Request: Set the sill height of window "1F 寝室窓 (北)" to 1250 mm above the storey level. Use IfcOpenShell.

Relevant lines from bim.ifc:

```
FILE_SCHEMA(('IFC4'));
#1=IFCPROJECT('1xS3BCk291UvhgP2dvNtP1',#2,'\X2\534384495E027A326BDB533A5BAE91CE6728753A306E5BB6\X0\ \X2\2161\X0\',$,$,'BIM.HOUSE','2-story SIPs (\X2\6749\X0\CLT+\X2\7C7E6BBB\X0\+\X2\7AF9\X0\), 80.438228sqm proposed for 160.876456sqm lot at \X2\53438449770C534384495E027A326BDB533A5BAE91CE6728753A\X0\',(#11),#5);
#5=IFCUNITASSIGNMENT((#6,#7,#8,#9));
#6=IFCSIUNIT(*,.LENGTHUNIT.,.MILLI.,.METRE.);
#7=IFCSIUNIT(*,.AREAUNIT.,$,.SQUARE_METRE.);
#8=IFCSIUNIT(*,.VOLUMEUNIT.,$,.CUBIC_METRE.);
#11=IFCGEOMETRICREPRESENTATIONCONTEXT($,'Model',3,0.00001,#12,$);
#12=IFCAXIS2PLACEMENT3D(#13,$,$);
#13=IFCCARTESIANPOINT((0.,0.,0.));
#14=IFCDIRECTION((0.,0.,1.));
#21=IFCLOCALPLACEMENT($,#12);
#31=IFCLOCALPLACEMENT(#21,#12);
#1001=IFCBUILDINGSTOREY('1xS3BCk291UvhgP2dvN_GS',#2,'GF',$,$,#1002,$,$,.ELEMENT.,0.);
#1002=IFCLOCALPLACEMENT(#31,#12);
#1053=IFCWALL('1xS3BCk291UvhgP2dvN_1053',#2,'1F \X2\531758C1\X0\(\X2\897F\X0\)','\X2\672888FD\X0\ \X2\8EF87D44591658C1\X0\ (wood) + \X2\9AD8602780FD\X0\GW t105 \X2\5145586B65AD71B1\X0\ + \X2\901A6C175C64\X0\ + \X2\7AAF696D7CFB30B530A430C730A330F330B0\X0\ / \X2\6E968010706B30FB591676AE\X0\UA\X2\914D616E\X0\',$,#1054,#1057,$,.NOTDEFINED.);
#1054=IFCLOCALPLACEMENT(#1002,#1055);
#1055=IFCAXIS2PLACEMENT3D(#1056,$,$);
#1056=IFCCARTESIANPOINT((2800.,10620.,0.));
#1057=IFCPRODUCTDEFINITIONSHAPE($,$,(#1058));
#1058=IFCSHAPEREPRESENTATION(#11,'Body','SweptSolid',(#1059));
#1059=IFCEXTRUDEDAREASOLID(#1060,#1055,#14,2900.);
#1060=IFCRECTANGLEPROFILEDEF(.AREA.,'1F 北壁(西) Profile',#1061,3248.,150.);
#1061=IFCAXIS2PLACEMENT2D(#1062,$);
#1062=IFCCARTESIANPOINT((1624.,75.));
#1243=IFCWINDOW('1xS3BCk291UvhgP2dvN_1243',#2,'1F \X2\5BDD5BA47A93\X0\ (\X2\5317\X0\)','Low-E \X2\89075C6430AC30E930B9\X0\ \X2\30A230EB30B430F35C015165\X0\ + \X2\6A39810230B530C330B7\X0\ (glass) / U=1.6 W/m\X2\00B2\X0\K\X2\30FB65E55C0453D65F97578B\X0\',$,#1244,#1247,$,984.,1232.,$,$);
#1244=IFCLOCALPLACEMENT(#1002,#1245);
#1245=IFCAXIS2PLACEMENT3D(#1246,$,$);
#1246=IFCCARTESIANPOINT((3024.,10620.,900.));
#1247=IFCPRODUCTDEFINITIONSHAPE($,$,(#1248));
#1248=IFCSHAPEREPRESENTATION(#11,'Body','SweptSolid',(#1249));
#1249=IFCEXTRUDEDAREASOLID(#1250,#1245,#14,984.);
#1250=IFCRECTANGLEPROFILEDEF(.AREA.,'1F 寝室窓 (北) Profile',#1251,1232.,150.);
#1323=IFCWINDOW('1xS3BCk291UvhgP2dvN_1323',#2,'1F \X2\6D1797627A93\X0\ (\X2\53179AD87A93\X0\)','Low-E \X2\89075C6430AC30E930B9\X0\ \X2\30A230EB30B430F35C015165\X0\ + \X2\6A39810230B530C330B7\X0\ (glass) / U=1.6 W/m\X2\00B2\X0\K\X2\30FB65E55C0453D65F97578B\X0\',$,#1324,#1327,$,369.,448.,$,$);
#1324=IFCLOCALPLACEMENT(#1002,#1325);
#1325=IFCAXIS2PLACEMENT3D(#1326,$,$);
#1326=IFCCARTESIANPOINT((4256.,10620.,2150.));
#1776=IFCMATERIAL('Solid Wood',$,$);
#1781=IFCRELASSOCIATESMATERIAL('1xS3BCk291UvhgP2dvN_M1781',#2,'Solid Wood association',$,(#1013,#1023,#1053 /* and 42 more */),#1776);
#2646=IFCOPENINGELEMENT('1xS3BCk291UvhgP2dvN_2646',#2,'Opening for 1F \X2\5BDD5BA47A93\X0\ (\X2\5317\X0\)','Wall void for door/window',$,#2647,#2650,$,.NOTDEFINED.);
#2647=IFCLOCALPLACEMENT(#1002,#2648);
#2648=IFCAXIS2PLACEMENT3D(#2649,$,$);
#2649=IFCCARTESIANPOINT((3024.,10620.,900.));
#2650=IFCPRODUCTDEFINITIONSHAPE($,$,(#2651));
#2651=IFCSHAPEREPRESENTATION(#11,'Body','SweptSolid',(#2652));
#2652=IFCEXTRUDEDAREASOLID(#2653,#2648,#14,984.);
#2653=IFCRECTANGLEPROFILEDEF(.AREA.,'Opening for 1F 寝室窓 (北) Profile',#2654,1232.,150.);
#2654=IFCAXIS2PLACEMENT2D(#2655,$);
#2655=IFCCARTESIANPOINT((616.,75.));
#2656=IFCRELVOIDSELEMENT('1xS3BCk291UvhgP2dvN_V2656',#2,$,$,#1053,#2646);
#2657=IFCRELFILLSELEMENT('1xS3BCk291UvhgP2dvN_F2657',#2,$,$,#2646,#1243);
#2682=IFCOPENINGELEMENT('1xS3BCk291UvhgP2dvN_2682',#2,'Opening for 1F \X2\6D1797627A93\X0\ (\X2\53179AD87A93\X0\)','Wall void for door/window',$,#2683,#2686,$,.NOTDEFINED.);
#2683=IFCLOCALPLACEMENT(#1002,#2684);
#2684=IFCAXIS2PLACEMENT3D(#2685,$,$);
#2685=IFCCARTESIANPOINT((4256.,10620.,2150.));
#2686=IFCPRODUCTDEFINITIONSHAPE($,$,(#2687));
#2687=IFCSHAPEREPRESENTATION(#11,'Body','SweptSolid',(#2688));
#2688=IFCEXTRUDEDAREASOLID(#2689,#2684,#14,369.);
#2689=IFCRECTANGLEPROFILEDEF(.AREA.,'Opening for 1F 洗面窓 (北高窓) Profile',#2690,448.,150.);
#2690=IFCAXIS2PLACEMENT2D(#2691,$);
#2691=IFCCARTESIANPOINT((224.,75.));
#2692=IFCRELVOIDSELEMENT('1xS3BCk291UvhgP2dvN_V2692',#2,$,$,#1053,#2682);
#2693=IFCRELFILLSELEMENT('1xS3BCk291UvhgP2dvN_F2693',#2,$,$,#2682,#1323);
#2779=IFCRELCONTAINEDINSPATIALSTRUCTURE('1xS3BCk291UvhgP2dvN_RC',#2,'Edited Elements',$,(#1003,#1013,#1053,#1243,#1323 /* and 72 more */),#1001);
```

```python
import numpy as np
import ifcopenshell
import ifcopenshell.api.geometry
import ifcopenshell.geom
import ifcopenshell.util.element
import ifcopenshell.util.placement
import ifcopenshell.util.shape
import ifcopenshell.util.unit

model = ifcopenshell.open("bim.ifc")
unit_scale = ifcopenshell.util.unit.calculate_unit_scale(model)

window = model.by_guid("1xS3BCk291UvhgP2dvN_1243")
opening = window.FillsVoids[0].RelatingOpeningElement
storey = ifcopenshell.util.element.get_container(window, ifc_class="IfcBuildingStorey")
level = ifcopenshell.util.placement.get_local_placement(storey.ObjectPlacement)[2, 3]

# The opening's origin need not be at the sill, so measure its lowest point.
shape = ifcopenshell.geom.create_shape(ifcopenshell.geom.settings(), opening)
bottom = ifcopenshell.util.shape.get_shape_bottom_elevation(shape, shape.geometry) / unit_scale
dz = level + 1.25 / unit_scale - bottom

shift = np.array([0.0, 0.0, dz])
# The window is not placed relative to its opening, so move both.
for product in (opening, window):
    matrix = ifcopenshell.util.placement.get_local_placement(product.ObjectPlacement)
    matrix[:3, 3] += shift
    ifcopenshell.api.geometry.edit_object_placement(model, product=product, matrix=matrix, is_si=False)

print(f"moved by {dz * unit_scale:+.3f} m")

model.write("bim_rev.ifc")
```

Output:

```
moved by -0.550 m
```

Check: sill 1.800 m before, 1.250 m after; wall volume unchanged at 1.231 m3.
